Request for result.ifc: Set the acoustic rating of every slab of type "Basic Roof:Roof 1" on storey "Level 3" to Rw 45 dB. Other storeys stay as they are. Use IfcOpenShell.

First a look at what the model holds.

```python
import ifcopenshell
import ifcopenshell.util.element

model = ifcopenshell.open("result.ifc")
print(model.schema)
storey = next(s for s in model.by_type("IfcBuildingStorey") if s.Name == "Level 3")
slabs = [e for e in ifcopenshell.util.element.get_decomposition(storey) if e.is_a("IfcSlab")]
seen = {}
for e in slabs:
    element_type = ifcopenshell.util.element.get_type(e)
    key = (element_type.Name if element_type != e and element_type else None, ifcopenshell.util.element.get_pset(e, "Pset_SlabCommon", "AcousticRating"))
    seen[key] = seen.get(key, 0) + 1
for (name, value), count in sorted(seen.items(), key=str):
    print(count, "x", name, "|", value)
```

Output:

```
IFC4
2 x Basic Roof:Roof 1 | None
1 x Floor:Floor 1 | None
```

```python
import ifcopenshell
import ifcopenshell.api.pset
import ifcopenshell.util.element

model = ifcopenshell.open("result.ifc")

storey = next(s for s in model.by_type("IfcBuildingStorey") if s.Name == "Level 3")
slabs = [e for e in ifcopenshell.util.element.get_decomposition(storey) if e.is_a("IfcSlab")]

count = 0
for e in slabs:
    element_type = ifcopenshell.util.element.get_type(e)
    if element_type in (None, e) or element_type.Name != "Basic Roof:Roof 1":
        continue
    # add_pset returns the element's existing set when there is one.
    pset = ifcopenshell.api.pset.add_pset(model, product=e, name="Pset_SlabCommon")
    ifcopenshell.api.pset.edit_pset(model, pset=pset, properties={"AcousticRating": "Rw 45 dB"})
    count += 1

print(count, "slabs updated")

model.write("result_updated.ifc")
```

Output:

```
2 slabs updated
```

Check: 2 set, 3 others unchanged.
